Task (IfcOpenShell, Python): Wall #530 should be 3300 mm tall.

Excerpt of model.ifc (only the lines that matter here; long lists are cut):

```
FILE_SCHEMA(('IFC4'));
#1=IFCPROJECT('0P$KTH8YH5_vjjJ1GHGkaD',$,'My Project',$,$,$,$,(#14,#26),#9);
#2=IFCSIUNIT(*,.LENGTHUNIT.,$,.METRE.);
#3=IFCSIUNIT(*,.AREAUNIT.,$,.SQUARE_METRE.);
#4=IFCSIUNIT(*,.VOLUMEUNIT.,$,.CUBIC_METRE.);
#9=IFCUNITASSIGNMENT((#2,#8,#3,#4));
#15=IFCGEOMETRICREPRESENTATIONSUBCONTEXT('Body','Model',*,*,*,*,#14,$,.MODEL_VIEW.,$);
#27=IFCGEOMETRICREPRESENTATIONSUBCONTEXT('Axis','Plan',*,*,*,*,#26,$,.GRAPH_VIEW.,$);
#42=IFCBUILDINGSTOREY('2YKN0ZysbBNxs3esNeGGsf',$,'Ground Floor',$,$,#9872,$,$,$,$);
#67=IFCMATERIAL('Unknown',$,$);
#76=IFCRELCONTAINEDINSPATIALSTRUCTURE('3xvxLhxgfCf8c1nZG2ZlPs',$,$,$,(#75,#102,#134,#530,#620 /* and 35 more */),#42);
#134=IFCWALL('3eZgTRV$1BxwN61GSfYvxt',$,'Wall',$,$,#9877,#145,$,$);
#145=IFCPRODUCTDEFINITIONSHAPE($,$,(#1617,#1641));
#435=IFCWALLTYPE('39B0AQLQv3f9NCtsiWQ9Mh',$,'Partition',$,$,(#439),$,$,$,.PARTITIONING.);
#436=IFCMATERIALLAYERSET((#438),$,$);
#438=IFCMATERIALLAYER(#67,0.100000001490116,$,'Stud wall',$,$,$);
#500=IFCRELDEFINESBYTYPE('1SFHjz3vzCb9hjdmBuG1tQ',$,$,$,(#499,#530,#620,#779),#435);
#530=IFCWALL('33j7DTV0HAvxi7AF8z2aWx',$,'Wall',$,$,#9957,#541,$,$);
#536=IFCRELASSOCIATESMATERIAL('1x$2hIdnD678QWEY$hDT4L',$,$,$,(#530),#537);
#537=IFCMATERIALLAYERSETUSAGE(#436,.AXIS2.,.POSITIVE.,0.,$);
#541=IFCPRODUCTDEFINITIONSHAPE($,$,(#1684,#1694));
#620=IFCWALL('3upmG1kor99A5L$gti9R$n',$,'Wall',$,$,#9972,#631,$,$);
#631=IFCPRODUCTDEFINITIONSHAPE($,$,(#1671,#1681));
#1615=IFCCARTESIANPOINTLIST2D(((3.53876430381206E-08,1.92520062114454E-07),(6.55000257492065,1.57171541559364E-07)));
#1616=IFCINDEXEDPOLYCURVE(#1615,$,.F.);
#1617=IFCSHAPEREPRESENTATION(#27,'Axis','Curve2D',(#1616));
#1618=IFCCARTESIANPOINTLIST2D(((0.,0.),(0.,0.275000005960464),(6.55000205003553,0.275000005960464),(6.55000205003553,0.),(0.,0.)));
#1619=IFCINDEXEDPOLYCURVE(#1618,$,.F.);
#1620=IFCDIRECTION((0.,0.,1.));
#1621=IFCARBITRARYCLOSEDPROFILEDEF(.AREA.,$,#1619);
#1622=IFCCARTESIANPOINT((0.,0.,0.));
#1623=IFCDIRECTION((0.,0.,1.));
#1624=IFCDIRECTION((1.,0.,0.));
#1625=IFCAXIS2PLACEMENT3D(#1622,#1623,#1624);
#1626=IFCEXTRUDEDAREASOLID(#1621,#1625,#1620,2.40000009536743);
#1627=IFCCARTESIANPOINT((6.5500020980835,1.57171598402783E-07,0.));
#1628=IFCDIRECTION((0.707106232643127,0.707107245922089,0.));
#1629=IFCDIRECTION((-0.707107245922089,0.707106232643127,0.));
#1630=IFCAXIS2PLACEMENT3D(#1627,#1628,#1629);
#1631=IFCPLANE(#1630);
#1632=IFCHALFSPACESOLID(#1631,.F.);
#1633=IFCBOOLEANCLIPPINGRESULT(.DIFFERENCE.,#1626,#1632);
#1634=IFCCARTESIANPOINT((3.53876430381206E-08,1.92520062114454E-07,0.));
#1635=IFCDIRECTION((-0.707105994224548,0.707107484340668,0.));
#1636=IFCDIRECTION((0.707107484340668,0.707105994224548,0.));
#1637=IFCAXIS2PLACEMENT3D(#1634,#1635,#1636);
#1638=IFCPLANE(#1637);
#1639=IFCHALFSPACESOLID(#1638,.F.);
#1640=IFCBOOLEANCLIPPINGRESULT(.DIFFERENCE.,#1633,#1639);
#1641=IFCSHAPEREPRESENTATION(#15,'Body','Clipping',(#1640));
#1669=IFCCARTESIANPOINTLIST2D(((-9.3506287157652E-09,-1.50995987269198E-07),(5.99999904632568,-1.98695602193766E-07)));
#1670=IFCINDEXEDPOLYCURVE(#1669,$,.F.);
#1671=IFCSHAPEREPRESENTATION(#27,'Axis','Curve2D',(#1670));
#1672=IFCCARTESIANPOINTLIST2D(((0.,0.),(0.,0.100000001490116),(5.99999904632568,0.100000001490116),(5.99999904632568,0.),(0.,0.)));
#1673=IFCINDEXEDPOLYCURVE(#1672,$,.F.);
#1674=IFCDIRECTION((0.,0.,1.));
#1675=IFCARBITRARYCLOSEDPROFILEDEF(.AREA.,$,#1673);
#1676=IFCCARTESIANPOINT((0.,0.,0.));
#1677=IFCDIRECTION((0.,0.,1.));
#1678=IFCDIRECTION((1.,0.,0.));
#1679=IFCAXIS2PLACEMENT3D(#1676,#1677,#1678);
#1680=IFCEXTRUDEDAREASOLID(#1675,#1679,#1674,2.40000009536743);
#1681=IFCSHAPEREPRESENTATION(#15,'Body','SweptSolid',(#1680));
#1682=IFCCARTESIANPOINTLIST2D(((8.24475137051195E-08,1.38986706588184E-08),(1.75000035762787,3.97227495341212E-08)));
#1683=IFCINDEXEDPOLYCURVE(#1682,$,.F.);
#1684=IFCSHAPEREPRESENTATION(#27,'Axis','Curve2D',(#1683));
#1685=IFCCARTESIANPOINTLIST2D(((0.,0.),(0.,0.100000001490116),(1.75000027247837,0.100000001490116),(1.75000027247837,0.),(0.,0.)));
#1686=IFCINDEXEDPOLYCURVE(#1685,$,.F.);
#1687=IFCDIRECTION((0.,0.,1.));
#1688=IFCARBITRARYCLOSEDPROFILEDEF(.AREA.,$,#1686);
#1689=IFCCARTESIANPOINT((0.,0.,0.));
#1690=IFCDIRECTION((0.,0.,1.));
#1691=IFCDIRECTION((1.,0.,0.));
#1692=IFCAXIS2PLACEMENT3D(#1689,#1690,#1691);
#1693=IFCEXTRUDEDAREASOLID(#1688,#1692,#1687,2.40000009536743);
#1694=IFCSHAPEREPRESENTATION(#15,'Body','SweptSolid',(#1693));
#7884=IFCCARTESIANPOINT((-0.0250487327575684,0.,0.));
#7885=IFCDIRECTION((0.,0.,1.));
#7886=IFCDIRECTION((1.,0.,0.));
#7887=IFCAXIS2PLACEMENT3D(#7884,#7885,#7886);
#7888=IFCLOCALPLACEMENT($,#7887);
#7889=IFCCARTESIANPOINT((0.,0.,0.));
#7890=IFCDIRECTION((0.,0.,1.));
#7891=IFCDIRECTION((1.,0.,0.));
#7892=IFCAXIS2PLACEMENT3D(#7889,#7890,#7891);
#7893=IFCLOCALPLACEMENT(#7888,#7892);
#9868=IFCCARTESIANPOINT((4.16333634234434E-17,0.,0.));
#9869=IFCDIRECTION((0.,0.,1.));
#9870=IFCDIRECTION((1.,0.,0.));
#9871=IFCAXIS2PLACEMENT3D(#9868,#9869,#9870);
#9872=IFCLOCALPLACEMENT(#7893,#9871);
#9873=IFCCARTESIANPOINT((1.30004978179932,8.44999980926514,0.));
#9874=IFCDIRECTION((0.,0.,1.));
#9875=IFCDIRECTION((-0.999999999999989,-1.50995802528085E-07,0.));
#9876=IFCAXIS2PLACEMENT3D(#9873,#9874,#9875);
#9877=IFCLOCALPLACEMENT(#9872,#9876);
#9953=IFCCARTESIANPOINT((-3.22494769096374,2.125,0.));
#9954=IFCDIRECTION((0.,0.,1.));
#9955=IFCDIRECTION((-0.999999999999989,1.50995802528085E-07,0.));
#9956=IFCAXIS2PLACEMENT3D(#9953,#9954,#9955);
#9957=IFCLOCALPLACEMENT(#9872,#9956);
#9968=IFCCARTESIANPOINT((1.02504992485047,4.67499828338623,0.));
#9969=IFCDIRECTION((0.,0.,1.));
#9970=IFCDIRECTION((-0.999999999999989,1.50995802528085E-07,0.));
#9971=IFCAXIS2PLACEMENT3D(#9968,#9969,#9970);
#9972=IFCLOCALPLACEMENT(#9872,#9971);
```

```python
import ifcopenshell
import ifcopenshell.geom
import ifcopenshell.util.representation
import ifcopenshell.util.shape
import ifcopenshell.util.unit

model = ifcopenshell.open("model.ifc")
unit_scale = ifcopenshell.util.unit.calculate_unit_scale(model)
settings = ifcopenshell.geom.settings()


def volume(element):
    """Net volume in cubic metres, openings subtracted."""
    shape = ifcopenshell.geom.create_shape(settings, element)
    return ifcopenshell.util.shape.get_volume(shape.geometry)


wall = model.by_guid("33j7DTV0HAvxi7AF8z2aWx")
before = volume(wall)

body = ifcopenshell.util.representation.get_representation(wall, "Model", "Body")
solid = body.Items[0]
old_height = solid.Depth
solid.Depth = 3.3 / unit_scale
after = volume(wall)

print(f"height {old_height:g} -> {solid.Depth:g}, volume {before:.3f} -> {after:.3f} m3")

model.write("model_rev.ifc")
```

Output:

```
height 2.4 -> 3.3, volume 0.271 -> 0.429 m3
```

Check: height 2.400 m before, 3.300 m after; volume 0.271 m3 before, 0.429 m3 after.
